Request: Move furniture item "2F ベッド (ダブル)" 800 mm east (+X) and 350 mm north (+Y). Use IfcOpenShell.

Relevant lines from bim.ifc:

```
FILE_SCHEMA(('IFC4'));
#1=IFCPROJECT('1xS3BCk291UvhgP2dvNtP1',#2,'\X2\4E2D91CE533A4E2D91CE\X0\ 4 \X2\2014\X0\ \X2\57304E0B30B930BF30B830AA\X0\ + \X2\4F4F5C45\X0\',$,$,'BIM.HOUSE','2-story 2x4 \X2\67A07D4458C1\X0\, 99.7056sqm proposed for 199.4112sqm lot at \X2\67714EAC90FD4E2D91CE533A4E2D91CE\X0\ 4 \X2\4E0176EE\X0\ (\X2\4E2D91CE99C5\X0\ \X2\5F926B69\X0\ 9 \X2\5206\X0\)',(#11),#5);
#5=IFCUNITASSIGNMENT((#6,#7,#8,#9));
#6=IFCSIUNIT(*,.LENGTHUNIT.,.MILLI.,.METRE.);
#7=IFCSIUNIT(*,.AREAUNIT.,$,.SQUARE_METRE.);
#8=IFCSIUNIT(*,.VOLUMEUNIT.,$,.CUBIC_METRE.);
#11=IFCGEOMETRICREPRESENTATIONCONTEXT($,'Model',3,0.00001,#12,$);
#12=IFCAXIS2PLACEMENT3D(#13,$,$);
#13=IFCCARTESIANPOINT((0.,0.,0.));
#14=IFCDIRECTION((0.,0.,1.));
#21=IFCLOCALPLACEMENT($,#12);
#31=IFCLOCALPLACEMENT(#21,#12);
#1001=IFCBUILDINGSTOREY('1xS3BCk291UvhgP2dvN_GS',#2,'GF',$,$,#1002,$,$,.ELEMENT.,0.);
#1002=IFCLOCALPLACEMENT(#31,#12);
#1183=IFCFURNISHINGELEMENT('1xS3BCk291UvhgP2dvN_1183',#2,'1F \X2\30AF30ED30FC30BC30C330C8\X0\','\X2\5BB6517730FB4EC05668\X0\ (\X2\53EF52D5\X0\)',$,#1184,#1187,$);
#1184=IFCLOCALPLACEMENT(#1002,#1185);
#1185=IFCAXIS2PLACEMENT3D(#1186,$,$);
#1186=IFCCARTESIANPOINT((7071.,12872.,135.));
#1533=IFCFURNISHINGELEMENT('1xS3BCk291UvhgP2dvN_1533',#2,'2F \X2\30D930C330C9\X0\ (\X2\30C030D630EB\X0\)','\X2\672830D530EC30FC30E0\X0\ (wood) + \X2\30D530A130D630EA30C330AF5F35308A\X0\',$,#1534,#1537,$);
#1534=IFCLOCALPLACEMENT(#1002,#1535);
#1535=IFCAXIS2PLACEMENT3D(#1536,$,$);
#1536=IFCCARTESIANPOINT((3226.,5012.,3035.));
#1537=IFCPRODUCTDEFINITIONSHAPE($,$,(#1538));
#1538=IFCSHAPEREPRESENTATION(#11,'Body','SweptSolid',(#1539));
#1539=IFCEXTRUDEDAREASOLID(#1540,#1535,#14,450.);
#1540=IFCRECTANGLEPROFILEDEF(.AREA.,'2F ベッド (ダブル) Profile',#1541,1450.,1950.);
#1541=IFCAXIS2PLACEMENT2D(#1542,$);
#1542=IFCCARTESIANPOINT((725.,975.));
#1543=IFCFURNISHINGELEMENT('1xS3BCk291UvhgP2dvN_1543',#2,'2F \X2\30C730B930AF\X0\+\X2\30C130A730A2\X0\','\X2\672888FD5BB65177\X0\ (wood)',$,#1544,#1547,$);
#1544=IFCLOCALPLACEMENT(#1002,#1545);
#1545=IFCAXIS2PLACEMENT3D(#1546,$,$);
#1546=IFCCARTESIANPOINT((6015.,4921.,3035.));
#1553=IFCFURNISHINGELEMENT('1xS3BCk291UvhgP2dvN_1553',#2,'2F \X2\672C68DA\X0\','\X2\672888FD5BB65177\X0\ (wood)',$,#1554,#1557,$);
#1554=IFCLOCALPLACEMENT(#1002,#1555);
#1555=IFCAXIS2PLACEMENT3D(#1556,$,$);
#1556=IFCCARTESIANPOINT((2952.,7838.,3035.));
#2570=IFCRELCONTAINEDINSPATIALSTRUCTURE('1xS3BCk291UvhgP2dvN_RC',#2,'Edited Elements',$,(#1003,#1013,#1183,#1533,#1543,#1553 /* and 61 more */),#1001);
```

```python
import ifcopenshell
import ifcopenshell.api.geometry
import ifcopenshell.util.placement
import ifcopenshell.util.unit

model = ifcopenshell.open("bim.ifc")
unit_scale = ifcopenshell.util.unit.calculate_unit_scale(model)

item = model.by_guid("1xS3BCk291UvhgP2dvN_1533")
matrix = ifcopenshell.util.placement.get_local_placement(item.ObjectPlacement)
matrix[0, 3] += 0.8 / unit_scale
matrix[1, 3] += 0.35 / unit_scale
ifcopenshell.api.geometry.edit_object_placement(model, product=item, matrix=matrix, is_si=False)

print(ifcopenshell.util.placement.get_local_placement(item.ObjectPlacement).round(3) + 0.0)

model.write("bim_v2.ifc")
```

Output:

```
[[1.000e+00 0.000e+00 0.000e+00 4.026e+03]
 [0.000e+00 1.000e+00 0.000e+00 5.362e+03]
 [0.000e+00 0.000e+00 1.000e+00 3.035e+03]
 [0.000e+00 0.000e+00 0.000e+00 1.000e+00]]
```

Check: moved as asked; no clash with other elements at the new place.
